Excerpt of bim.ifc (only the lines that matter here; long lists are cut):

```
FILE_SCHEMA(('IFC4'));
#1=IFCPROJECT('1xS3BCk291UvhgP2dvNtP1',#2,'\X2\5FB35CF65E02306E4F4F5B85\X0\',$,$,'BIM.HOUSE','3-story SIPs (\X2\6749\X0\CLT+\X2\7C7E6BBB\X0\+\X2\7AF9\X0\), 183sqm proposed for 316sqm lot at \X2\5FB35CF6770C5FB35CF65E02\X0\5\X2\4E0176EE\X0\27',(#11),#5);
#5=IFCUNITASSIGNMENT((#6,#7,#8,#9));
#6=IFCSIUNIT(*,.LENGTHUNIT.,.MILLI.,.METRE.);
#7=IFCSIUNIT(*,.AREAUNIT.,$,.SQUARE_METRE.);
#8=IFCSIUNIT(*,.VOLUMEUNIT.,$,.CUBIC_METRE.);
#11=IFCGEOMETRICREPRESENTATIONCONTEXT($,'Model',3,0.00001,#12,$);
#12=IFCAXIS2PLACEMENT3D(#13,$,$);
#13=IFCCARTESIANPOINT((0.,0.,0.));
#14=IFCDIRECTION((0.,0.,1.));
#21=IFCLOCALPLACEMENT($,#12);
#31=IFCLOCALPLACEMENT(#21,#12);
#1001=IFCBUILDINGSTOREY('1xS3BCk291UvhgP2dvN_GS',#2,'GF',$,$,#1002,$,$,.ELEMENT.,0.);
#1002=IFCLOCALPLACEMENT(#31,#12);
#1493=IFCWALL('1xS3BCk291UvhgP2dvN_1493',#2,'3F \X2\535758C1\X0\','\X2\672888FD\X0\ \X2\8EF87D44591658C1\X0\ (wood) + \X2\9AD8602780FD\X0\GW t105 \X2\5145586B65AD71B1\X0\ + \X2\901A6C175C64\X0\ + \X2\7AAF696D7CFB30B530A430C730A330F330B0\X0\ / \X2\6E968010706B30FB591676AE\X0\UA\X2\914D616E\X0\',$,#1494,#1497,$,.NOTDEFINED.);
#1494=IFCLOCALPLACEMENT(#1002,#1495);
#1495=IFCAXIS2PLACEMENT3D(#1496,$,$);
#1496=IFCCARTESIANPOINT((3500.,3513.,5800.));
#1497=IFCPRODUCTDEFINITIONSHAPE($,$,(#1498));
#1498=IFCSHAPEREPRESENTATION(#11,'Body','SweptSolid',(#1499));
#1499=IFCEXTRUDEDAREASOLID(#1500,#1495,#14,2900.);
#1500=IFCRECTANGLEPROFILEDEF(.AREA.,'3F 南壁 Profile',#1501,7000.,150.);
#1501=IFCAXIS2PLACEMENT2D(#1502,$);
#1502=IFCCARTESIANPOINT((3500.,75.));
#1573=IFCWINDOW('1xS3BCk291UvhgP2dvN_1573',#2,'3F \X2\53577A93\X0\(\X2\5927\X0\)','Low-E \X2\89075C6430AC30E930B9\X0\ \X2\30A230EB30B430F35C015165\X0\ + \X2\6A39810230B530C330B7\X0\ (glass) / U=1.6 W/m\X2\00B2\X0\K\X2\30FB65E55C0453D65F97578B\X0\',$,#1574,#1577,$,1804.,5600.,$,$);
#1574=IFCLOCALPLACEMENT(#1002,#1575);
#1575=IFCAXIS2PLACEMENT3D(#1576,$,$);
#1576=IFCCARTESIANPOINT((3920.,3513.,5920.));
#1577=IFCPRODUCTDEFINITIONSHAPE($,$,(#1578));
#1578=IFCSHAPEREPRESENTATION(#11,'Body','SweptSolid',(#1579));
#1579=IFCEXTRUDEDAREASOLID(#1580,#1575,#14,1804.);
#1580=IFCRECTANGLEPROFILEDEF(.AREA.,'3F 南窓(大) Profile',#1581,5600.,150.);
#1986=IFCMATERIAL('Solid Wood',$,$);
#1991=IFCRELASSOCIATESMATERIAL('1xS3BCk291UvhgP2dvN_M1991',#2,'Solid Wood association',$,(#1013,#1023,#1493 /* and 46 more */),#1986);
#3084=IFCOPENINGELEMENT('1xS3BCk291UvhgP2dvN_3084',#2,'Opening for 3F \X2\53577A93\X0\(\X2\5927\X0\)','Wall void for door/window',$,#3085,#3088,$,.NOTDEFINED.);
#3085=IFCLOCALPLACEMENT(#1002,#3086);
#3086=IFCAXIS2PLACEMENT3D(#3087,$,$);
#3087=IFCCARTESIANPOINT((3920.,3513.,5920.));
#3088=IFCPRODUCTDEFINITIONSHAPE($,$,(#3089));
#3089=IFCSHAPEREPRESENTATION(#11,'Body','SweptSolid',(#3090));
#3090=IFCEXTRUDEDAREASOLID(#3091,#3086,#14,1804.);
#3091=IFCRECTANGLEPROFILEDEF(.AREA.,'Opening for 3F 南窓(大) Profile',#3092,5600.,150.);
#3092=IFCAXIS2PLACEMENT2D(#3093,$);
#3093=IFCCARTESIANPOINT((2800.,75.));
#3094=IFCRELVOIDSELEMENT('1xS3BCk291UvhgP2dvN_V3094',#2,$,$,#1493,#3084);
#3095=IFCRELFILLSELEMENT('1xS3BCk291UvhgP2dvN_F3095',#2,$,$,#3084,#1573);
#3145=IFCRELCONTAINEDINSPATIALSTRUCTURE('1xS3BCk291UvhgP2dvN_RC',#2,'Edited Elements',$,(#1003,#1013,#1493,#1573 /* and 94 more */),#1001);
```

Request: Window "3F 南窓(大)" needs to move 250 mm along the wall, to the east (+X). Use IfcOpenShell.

```python
import ifcopenshell
import ifcopenshell.api.geometry
import ifcopenshell.util.placement
import ifcopenshell.util.unit

model = ifcopenshell.open("bim.ifc")
unit_scale = ifcopenshell.util.unit.calculate_unit_scale(model)

window = model.by_id(1573)
opening = window.FillsVoids[0].RelatingOpeningElement
wall = opening.VoidsElements[0].RelatingBuildingElement

wall_matrix = ifcopenshell.util.placement.get_local_placement(wall.ObjectPlacement)
shift = wall_matrix[:3, 0] * 0.25 / unit_scale
before = ifcopenshell.util.placement.get_local_placement(window.ObjectPlacement)[:3, 3].copy()

# The window is not placed relative to its opening, so move both.
for product in (opening, window):
    matrix = ifcopenshell.util.placement.get_local_placement(product.ObjectPlacement)
    matrix[:3, 3] += shift
    ifcopenshell.api.geometry.edit_object_placement(model, product=product, matrix=matrix, is_si=False)

after = ifcopenshell.util.placement.get_local_placement(window.ObjectPlacement)[:3, 3]
print("window moved by", (after - before).round(3) + 0.0)

model.write("bim_rev.ifc")
```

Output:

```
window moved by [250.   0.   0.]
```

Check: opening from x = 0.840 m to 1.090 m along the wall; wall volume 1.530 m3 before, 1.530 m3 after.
